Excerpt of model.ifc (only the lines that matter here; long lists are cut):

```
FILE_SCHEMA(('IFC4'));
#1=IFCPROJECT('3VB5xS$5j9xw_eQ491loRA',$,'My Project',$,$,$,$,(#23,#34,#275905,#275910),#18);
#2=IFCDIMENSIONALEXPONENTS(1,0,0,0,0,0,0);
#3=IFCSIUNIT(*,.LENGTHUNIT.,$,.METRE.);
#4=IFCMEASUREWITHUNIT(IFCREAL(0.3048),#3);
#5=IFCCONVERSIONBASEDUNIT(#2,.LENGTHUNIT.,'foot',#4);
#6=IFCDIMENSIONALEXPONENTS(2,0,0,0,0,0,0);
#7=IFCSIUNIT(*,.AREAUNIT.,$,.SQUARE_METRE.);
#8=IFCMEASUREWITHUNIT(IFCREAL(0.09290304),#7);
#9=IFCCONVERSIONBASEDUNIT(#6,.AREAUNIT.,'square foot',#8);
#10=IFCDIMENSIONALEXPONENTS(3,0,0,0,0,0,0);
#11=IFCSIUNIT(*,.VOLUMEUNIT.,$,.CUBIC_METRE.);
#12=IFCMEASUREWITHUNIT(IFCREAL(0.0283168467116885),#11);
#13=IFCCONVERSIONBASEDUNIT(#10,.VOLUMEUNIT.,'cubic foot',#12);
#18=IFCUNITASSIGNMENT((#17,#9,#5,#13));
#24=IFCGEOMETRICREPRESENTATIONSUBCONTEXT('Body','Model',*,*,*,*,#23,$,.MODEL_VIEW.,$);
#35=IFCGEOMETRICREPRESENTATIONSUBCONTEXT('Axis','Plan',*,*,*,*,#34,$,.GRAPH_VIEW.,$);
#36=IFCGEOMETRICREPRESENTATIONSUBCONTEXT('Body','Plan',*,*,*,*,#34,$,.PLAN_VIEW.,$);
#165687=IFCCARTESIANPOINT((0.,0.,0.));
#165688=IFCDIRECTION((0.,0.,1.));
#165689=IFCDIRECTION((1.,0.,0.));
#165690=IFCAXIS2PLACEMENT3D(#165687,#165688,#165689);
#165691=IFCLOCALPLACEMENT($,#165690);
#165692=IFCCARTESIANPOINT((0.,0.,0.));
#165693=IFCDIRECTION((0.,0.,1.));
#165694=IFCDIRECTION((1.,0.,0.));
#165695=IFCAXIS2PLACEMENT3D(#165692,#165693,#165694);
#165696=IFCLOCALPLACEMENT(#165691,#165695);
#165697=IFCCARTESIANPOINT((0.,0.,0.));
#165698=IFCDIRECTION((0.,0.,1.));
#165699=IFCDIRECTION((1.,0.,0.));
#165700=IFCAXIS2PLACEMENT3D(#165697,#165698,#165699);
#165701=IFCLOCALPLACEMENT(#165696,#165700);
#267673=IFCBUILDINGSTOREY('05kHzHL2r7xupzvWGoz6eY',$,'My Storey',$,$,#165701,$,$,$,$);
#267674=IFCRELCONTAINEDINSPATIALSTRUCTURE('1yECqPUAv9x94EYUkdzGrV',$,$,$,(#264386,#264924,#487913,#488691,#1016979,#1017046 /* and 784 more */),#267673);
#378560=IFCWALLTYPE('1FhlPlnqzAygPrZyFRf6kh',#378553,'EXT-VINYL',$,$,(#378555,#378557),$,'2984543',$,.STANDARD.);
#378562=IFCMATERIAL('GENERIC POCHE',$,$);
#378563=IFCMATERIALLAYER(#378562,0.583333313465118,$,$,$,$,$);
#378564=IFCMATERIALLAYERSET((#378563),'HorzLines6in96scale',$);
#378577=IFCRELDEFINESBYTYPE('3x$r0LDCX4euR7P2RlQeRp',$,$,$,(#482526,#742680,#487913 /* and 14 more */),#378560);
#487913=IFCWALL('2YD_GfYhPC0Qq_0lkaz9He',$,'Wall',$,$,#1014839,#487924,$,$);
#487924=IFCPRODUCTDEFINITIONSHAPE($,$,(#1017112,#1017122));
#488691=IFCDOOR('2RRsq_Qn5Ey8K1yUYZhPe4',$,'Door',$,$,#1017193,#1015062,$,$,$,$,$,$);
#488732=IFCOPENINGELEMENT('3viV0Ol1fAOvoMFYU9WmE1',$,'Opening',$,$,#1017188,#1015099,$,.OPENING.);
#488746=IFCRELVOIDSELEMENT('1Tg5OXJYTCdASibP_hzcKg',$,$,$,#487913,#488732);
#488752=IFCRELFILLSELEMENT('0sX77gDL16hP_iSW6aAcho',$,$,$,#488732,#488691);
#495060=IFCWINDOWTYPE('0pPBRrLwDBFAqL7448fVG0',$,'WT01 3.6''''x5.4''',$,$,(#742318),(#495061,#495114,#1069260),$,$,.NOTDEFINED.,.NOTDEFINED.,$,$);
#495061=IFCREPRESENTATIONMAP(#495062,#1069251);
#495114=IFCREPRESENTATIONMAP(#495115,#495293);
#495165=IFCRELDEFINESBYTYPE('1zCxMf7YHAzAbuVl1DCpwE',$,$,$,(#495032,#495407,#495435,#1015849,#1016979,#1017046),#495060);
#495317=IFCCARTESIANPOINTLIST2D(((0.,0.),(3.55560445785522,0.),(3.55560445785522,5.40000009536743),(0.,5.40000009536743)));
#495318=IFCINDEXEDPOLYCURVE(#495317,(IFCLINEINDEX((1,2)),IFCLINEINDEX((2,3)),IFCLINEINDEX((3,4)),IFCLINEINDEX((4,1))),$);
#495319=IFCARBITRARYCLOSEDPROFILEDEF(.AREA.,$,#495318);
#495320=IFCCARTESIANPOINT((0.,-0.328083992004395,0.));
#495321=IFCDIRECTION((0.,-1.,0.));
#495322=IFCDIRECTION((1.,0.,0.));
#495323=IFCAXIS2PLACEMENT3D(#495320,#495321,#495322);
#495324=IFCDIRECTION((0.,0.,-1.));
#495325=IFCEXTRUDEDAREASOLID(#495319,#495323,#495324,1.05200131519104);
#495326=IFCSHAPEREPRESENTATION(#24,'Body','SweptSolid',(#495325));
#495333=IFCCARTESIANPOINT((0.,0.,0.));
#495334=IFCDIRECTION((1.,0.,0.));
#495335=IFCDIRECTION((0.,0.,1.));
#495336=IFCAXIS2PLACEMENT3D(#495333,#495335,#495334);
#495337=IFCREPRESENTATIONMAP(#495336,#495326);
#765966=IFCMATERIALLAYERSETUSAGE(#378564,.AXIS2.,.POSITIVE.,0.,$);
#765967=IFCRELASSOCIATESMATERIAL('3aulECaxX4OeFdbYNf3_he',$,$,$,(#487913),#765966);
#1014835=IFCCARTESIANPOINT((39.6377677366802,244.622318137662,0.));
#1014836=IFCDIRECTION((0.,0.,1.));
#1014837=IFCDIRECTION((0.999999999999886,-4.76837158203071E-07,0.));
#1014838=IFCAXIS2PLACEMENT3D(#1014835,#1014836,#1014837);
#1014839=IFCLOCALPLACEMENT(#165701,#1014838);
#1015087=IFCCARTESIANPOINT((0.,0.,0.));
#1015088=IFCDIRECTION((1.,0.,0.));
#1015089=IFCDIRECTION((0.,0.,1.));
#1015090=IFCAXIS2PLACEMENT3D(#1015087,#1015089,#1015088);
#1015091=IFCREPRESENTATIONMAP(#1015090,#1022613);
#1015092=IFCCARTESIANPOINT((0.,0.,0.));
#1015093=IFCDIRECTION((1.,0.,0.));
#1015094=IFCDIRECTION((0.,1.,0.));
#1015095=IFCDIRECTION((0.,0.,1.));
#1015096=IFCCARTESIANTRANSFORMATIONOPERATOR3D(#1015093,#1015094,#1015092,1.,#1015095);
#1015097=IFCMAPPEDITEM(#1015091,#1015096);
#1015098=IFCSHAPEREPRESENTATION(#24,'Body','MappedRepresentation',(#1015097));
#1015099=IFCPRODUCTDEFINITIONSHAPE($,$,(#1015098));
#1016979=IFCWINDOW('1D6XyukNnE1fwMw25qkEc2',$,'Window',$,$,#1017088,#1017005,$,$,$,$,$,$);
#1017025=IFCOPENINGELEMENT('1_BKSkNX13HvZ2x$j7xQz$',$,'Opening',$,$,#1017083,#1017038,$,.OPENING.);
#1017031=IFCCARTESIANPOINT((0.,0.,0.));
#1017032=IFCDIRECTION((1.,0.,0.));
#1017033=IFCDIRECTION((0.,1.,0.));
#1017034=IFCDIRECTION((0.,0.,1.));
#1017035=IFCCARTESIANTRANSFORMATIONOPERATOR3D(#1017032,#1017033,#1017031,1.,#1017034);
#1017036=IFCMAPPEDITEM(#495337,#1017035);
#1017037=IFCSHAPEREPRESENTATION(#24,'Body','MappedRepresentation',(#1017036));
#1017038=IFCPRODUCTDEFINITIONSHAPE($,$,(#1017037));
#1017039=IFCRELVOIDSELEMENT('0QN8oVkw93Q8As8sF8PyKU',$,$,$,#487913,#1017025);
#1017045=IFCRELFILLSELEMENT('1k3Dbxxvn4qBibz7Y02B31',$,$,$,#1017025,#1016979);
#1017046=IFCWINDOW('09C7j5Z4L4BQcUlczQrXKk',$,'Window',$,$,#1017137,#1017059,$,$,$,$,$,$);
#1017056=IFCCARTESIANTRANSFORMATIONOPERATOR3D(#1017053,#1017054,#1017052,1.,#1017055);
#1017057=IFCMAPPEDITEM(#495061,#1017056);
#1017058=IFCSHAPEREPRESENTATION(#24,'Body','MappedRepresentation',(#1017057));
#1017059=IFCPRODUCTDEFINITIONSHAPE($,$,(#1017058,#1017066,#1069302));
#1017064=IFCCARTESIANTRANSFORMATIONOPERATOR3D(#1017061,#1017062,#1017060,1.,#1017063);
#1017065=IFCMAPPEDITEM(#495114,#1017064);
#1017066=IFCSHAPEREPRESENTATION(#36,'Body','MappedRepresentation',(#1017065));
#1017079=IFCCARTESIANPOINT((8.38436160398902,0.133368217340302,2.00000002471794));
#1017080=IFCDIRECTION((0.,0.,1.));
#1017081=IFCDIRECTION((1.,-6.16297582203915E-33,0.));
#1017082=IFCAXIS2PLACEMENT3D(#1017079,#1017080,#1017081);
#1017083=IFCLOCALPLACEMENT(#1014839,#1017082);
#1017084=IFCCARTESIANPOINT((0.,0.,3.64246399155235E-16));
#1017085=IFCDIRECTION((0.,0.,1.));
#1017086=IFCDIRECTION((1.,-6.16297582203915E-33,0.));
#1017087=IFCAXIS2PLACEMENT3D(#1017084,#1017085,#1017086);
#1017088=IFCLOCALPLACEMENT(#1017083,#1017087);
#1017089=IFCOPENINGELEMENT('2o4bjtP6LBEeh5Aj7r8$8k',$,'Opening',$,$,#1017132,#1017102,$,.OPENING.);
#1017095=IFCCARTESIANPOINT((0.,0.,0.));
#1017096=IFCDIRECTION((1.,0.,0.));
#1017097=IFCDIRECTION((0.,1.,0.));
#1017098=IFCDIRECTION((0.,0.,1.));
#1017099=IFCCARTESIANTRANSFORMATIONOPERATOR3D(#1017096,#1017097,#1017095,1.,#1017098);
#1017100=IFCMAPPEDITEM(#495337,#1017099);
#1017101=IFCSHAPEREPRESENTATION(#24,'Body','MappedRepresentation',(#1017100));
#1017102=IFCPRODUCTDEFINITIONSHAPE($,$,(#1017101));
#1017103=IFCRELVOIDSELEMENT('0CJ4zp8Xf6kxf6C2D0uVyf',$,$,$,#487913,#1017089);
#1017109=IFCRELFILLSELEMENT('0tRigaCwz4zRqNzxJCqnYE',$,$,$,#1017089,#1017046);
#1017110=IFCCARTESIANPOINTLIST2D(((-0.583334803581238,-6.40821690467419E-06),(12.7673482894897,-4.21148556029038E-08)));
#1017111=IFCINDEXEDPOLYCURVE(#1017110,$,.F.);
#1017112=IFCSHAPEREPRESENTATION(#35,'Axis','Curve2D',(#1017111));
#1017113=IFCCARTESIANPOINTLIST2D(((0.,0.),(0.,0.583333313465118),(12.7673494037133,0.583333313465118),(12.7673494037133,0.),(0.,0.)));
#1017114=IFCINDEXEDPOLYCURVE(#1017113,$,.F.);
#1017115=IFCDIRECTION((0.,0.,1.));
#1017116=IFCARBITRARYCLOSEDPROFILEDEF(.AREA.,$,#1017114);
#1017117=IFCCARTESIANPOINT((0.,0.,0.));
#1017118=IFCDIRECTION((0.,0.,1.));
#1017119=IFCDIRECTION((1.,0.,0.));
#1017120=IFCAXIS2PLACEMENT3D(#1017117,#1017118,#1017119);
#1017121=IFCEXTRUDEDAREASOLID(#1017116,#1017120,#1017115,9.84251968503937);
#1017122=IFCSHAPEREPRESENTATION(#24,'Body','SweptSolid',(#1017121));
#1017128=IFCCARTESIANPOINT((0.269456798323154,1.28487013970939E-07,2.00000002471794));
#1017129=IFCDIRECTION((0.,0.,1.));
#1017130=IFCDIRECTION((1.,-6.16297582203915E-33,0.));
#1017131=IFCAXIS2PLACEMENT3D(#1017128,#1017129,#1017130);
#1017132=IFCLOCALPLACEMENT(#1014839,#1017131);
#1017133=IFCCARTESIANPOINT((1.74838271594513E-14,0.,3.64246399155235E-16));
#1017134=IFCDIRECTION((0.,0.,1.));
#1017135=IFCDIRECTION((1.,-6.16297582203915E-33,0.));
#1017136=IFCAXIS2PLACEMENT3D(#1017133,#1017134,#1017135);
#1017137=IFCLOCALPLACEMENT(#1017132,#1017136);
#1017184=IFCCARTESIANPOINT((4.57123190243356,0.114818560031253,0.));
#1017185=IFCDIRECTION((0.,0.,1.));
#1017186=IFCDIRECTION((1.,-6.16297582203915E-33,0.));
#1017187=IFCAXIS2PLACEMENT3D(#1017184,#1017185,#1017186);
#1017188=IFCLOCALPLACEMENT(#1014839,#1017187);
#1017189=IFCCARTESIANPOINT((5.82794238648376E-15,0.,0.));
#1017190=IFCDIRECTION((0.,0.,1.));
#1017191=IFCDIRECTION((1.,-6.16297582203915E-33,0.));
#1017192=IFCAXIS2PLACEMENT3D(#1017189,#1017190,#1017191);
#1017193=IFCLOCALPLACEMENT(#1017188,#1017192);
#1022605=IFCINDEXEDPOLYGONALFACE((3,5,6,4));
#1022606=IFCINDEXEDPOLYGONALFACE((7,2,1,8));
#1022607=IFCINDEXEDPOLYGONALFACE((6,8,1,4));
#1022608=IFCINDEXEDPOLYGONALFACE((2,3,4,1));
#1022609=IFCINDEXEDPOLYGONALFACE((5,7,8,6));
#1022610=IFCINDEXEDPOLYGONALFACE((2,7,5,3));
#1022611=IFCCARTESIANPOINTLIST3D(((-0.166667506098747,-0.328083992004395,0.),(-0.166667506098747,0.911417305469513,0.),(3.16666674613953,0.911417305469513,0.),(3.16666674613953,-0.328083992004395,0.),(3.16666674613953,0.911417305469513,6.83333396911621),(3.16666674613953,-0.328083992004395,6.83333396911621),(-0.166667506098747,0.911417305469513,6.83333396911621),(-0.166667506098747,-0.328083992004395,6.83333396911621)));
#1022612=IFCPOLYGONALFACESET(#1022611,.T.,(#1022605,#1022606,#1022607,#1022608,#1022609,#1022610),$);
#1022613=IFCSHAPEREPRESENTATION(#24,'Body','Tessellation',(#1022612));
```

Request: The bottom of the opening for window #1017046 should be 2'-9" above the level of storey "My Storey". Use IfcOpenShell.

```python
import numpy as np
import ifcopenshell
import ifcopenshell.api.geometry
import ifcopenshell.geom
import ifcopenshell.util.element
import ifcopenshell.util.placement
import ifcopenshell.util.shape
import ifcopenshell.util.unit

model = ifcopenshell.open("model.ifc")
unit_scale = ifcopenshell.util.unit.calculate_unit_scale(model)

window = model.by_id(1017046)
opening = window.FillsVoids[0].RelatingOpeningElement
storey = ifcopenshell.util.element.get_container(window, ifc_class="IfcBuildingStorey")
level = ifcopenshell.util.placement.get_local_placement(storey.ObjectPlacement)[2, 3]

# The opening's origin need not be at the sill, so measure its lowest point.
shape = ifcopenshell.geom.create_shape(ifcopenshell.geom.settings(), opening)
bottom = ifcopenshell.util.shape.get_shape_bottom_elevation(shape, shape.geometry) / unit_scale
dz = level + 33 * 0.0254 / unit_scale - bottom

shift = np.array([0.0, 0.0, dz])
# The window is placed relative to its opening, so it follows when the opening moves.
matrix = ifcopenshell.util.placement.get_local_placement(opening.ObjectPlacement)
matrix[:3, 3] += shift
ifcopenshell.api.geometry.edit_object_placement(
    model, product=opening, matrix=matrix, is_si=False, should_transform_children=True
)

print(f"moved by {dz * unit_scale:+.3f} m")

model.write("model_updated.ifc")
```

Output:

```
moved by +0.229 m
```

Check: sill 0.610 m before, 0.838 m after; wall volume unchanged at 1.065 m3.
